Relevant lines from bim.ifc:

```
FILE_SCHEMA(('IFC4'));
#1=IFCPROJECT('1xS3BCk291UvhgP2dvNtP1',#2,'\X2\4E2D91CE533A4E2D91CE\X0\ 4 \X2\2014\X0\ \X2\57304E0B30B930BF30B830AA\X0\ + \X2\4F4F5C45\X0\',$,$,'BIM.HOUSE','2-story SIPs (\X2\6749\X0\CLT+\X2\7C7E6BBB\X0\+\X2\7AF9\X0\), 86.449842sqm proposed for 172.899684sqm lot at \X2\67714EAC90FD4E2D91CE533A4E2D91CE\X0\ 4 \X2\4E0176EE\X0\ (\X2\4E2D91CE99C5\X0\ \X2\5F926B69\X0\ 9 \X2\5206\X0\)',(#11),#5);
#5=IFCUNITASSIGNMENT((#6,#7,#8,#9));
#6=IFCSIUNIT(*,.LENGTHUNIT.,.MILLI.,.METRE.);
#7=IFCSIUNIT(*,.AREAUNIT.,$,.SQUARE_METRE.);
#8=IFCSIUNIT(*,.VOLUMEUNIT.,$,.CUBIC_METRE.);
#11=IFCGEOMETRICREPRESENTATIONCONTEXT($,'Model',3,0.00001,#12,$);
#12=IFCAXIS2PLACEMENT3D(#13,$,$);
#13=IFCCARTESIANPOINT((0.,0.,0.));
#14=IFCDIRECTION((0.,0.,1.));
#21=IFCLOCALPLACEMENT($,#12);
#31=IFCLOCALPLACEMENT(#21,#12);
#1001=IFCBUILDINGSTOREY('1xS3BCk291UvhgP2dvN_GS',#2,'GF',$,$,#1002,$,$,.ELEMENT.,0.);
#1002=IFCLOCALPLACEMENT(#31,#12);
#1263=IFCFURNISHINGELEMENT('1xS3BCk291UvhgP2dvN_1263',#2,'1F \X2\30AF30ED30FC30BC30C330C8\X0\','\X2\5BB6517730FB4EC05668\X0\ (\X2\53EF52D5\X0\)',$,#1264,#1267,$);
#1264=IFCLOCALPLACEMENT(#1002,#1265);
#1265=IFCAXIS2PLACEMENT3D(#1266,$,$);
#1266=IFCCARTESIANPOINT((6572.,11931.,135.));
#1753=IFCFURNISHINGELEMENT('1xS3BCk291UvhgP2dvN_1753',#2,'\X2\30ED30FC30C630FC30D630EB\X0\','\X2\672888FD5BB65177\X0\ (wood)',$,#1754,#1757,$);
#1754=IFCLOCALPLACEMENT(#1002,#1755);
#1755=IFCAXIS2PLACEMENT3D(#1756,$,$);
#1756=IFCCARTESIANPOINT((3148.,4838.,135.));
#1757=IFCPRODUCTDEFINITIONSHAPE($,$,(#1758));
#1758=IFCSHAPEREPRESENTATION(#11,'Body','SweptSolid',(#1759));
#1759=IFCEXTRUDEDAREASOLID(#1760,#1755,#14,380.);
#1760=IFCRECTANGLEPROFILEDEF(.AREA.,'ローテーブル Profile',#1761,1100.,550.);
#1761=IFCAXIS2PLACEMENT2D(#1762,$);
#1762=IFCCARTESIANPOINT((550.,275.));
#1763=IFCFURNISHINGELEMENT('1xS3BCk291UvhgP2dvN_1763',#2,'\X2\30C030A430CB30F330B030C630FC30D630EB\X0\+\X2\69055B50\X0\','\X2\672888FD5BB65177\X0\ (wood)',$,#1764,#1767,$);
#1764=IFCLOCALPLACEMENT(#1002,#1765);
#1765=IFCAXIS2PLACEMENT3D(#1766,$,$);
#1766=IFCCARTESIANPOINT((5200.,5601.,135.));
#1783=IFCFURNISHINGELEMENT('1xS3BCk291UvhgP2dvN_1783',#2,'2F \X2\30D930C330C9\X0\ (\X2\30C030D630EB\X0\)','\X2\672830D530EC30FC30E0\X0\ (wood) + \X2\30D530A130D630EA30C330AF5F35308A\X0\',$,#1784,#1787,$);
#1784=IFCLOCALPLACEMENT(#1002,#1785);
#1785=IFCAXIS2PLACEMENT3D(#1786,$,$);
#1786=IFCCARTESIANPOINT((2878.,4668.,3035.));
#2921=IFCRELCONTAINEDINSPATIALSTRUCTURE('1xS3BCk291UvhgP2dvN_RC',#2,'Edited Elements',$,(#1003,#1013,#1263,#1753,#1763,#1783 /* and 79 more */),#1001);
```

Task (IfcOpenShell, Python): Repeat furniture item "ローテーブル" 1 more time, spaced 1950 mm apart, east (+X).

```python
import numpy as np
import ifcopenshell
import ifcopenshell.api.geometry
import ifcopenshell.api.root
import ifcopenshell.util.element
import ifcopenshell.util.placement
import ifcopenshell.util.unit

model = ifcopenshell.open("bim.ifc")
unit_scale = ifcopenshell.util.unit.calculate_unit_scale(model)


def reuse_history(source, copy):
    """copy_class also copies each property set's owner history, people and application; keep the originals."""
    for rel in copy.IsDefinedBy:
        if rel.is_a("IfcRelDefinesByProperties") and (history := rel.RelatingPropertyDefinition.OwnerHistory):
            rel.RelatingPropertyDefinition.OwnerHistory = source.OwnerHistory
            ifcopenshell.util.element.remove_deep2(model, history)


source = model.by_guid("1xS3BCk291UvhgP2dvN_1753")
base = ifcopenshell.util.placement.get_local_placement(source.ObjectPlacement)
step = np.array([1.0, 0.0, 0.0]) * 1.95 / unit_scale

for i in range(1, 2):
    copy = ifcopenshell.api.root.copy_class(model, product=source)
    copy.Representation = ifcopenshell.util.element.copy_deep(
        model, source.Representation, exclude=["IfcGeometricRepresentationContext", "IfcRepresentationMap"]
    )
    reuse_history(source, copy)
    matrix = base.copy()
    matrix[:3, 3] += i * step
    print("added at", matrix[:3, 3].round(3) + 0.0)
    ifcopenshell.api.geometry.edit_object_placement(model, product=copy, matrix=matrix, is_si=False)

model.write("bim_rev.ifc")
```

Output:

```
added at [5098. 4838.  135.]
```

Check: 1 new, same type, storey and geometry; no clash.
